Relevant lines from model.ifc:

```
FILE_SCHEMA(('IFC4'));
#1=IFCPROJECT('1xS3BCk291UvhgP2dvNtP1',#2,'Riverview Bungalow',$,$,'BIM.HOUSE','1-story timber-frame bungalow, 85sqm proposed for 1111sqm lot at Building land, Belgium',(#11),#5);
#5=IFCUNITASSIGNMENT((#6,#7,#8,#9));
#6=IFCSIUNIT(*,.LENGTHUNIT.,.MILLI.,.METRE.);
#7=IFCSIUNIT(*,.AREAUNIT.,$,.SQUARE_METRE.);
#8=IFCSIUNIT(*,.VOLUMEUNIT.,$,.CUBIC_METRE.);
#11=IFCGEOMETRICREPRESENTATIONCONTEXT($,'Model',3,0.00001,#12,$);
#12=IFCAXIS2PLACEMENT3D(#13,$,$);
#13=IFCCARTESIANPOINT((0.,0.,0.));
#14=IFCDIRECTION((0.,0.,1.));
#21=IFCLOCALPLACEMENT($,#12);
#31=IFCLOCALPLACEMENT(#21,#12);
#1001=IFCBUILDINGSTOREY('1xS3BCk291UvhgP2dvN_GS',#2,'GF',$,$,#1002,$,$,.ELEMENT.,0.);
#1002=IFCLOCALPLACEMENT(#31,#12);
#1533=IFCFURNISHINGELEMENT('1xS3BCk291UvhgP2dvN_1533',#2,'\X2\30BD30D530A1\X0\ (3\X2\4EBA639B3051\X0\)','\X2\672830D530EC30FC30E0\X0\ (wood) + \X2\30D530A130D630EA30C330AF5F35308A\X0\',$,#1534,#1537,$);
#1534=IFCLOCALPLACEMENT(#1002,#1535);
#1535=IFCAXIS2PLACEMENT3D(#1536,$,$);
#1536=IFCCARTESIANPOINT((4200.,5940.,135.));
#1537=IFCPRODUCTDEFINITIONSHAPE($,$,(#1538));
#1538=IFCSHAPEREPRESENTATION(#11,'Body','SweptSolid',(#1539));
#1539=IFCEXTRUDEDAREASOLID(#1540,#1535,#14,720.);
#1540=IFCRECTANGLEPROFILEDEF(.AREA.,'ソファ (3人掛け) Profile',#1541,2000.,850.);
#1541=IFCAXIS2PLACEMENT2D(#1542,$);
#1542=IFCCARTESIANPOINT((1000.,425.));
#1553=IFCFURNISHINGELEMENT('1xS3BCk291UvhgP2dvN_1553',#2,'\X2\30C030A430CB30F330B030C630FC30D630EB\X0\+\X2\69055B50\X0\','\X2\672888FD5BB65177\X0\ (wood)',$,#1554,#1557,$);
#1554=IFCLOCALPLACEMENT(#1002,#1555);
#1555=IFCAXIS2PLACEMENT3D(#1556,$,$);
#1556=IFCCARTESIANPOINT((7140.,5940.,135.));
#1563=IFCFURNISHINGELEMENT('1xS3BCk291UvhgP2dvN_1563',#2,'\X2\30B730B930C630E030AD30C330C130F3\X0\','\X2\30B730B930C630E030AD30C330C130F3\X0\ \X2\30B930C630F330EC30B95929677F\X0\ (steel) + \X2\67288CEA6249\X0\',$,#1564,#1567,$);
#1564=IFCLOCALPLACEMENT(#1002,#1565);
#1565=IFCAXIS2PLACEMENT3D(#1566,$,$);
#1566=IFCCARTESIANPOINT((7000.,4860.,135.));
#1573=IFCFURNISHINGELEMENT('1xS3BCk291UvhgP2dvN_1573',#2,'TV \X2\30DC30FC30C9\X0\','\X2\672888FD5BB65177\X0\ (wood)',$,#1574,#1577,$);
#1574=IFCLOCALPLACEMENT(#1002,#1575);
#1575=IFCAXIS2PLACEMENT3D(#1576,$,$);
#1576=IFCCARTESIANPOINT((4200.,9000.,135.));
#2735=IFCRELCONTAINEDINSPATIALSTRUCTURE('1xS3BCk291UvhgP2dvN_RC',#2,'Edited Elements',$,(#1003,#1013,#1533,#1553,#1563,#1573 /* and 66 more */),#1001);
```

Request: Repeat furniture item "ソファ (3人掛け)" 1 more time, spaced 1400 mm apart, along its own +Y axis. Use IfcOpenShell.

```python
import ifcopenshell
import ifcopenshell.api.geometry
import ifcopenshell.api.root
import ifcopenshell.util.element
import ifcopenshell.util.placement
import ifcopenshell.util.unit

model = ifcopenshell.open("model.ifc")
unit_scale = ifcopenshell.util.unit.calculate_unit_scale(model)


def reuse_history(source, copy):
    """copy_class also copies each property set's owner history, people and application; keep the originals."""
    for rel in copy.IsDefinedBy:
        if rel.is_a("IfcRelDefinesByProperties") and (history := rel.RelatingPropertyDefinition.OwnerHistory):
            rel.RelatingPropertyDefinition.OwnerHistory = source.OwnerHistory
            ifcopenshell.util.element.remove_deep2(model, history)


source = model.by_guid("1xS3BCk291UvhgP2dvN_1533")
base = ifcopenshell.util.placement.get_local_placement(source.ObjectPlacement)
step = base[:3, 1] * 1.4 / unit_scale

for i in range(1, 2):
    copy = ifcopenshell.api.root.copy_class(model, product=source)
    copy.Representation = ifcopenshell.util.element.copy_deep(
        model, source.Representation, exclude=["IfcGeometricRepresentationContext", "IfcRepresentationMap"]
    )
    reuse_history(source, copy)
    matrix = base.copy()
    matrix[:3, 3] += i * step
    print("added at", matrix[:3, 3].round(3) + 0.0)
    ifcopenshell.api.geometry.edit_object_placement(model, product=copy, matrix=matrix, is_si=False)

model.write("model_v2.ifc")
```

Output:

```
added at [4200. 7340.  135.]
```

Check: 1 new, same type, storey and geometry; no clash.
